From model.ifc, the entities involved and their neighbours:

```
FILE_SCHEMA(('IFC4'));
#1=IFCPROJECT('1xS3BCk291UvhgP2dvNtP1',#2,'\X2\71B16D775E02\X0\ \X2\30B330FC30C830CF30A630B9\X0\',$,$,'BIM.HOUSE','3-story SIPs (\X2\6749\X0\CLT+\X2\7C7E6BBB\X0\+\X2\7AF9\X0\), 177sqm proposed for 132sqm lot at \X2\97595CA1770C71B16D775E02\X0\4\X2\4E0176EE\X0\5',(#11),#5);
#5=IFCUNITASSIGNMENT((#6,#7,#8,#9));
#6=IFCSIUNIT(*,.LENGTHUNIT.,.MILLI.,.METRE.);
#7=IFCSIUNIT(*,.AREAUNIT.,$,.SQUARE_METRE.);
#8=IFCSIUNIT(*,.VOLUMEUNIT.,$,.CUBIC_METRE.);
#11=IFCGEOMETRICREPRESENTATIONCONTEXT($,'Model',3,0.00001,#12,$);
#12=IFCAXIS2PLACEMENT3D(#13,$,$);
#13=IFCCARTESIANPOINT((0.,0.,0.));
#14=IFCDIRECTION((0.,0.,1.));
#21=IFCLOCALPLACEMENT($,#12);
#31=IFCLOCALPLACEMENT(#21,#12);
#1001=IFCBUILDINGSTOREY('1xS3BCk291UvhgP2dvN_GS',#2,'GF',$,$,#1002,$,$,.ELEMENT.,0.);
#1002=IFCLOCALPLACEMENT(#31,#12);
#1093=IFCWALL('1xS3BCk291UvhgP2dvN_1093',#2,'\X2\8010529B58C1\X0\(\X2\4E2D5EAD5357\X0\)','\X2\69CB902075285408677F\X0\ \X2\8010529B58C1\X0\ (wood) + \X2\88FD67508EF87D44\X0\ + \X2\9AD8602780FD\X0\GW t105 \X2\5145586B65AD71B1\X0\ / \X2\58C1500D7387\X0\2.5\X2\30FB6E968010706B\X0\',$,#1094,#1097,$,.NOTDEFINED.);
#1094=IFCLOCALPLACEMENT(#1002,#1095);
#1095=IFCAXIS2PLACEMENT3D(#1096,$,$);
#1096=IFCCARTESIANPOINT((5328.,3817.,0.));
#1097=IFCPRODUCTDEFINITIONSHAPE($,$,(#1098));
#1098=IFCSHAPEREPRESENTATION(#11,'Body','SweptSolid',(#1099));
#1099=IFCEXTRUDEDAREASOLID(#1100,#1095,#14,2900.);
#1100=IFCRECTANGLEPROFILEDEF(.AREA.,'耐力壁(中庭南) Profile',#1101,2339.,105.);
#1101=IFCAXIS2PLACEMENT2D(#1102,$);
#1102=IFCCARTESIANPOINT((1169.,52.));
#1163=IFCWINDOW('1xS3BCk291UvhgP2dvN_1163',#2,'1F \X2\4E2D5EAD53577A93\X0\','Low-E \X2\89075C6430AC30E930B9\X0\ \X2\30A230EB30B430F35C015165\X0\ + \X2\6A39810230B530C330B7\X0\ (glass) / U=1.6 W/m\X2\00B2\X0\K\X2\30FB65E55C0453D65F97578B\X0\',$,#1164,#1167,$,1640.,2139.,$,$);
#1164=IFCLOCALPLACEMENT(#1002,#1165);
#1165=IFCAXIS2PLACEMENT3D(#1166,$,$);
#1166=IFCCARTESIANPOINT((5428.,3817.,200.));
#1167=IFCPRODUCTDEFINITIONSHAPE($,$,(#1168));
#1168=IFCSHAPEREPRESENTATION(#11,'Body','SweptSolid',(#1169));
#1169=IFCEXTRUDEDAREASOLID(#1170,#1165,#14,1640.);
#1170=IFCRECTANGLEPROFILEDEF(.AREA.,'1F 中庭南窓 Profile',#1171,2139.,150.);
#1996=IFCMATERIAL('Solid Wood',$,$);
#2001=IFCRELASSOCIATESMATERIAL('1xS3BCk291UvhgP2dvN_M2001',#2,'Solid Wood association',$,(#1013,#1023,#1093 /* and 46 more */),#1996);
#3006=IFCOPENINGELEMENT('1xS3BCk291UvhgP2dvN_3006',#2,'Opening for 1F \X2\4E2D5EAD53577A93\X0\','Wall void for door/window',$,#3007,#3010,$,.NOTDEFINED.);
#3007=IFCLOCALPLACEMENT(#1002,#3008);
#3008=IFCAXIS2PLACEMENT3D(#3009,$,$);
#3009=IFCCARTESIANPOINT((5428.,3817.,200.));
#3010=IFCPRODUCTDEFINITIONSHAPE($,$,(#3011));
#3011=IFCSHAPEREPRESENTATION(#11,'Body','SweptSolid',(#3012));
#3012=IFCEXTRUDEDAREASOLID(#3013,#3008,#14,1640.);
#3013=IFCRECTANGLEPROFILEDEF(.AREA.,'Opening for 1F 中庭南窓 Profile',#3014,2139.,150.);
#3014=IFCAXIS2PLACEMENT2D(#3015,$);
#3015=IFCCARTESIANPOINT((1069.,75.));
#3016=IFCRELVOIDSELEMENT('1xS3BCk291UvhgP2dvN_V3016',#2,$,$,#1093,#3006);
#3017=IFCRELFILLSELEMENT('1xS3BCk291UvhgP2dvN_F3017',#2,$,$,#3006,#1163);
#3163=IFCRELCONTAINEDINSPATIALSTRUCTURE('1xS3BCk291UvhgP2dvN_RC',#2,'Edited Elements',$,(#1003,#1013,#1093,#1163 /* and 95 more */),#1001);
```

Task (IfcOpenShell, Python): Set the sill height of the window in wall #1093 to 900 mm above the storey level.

```python
import numpy as np
import ifcopenshell
import ifcopenshell.api.geometry
import ifcopenshell.geom
import ifcopenshell.util.element
import ifcopenshell.util.placement
import ifcopenshell.util.shape
import ifcopenshell.util.unit

model = ifcopenshell.open("model.ifc")
unit_scale = ifcopenshell.util.unit.calculate_unit_scale(model)

window = model.by_id(1163)
opening = window.FillsVoids[0].RelatingOpeningElement
storey = ifcopenshell.util.element.get_container(window, ifc_class="IfcBuildingStorey")
level = ifcopenshell.util.placement.get_local_placement(storey.ObjectPlacement)[2, 3]

# The opening's origin need not be at the sill, so measure its lowest point.
shape = ifcopenshell.geom.create_shape(ifcopenshell.geom.settings(), opening)
bottom = ifcopenshell.util.shape.get_shape_bottom_elevation(shape, shape.geometry) / unit_scale
dz = level + 0.9 / unit_scale - bottom

shift = np.array([0.0, 0.0, dz])
# The window is not placed relative to its opening, so move both.
for product in (opening, window):
    matrix = ifcopenshell.util.placement.get_local_placement(product.ObjectPlacement)
    matrix[:3, 3] += shift
    ifcopenshell.api.geometry.edit_object_placement(model, product=product, matrix=matrix, is_si=False)

print(f"moved by {dz * unit_scale:+.3f} m")

model.write("model_edited.ifc")
```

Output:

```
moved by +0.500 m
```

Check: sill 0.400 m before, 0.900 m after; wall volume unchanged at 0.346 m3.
